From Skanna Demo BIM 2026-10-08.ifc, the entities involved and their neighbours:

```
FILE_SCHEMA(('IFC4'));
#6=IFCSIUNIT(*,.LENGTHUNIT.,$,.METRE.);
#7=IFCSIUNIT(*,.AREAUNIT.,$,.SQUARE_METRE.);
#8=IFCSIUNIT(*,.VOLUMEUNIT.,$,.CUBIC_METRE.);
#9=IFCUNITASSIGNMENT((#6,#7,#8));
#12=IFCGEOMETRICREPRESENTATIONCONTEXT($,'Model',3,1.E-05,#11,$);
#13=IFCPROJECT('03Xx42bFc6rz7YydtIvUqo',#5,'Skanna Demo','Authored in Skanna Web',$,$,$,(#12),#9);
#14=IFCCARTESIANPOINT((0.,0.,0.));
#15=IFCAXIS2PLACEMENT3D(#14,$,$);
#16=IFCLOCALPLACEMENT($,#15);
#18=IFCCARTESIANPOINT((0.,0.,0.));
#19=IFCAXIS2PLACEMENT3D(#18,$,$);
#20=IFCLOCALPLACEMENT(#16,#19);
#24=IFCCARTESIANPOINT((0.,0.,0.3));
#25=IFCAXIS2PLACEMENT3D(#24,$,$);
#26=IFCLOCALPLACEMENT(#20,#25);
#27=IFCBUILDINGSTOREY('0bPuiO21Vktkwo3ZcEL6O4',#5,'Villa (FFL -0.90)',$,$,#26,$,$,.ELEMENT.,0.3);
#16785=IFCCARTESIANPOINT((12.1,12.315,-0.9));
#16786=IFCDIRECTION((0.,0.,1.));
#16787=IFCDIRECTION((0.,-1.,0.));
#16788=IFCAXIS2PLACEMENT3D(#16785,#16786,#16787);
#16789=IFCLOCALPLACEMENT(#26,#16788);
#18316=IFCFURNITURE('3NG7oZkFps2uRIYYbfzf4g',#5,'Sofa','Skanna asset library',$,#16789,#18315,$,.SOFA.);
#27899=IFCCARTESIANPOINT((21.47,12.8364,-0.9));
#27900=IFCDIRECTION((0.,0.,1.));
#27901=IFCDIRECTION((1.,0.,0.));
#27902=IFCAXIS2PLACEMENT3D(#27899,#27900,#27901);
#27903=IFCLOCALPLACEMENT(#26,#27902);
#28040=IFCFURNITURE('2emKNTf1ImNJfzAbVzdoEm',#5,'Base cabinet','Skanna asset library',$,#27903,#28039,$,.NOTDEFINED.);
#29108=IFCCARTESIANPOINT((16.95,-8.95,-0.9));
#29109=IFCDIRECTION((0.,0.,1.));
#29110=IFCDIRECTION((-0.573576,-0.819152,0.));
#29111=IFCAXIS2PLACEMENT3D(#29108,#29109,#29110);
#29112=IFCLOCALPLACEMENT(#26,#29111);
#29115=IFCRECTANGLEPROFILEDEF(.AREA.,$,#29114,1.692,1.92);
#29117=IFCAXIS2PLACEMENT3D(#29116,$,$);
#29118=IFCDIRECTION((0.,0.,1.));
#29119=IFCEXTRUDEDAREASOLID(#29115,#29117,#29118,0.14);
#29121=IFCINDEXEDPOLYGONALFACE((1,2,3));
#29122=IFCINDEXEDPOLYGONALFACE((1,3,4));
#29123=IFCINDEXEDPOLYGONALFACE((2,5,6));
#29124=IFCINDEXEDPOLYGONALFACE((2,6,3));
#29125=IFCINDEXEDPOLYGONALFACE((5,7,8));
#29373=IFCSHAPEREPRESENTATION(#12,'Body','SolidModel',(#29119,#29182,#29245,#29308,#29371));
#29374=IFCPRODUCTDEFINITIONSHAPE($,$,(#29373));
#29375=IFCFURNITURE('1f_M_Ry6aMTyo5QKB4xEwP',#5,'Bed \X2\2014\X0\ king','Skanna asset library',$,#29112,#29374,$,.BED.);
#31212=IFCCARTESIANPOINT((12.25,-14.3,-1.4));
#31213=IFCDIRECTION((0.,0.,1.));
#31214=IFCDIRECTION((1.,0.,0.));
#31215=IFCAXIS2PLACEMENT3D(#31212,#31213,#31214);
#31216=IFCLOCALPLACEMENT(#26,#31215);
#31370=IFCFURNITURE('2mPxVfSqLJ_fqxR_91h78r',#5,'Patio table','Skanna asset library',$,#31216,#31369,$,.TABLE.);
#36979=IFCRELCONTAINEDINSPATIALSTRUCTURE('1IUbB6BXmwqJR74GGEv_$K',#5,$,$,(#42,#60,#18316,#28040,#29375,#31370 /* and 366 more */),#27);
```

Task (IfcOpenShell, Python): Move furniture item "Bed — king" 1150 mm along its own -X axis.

```python
import ifcopenshell
import ifcopenshell.api.geometry
import ifcopenshell.util.placement
import ifcopenshell.util.unit

model = ifcopenshell.open("Skanna Demo BIM 2026-10-08.ifc")
unit_scale = ifcopenshell.util.unit.calculate_unit_scale(model)

item = model.by_id(29375)
matrix = ifcopenshell.util.placement.get_local_placement(item.ObjectPlacement)
matrix[:3, 3] -= matrix[:3, 0] * 1.15 / unit_scale
ifcopenshell.api.geometry.edit_object_placement(model, product=item, matrix=matrix, is_si=False)

print(ifcopenshell.util.placement.get_local_placement(item.ObjectPlacement).round(3) + 0.0)

model.write("Skanna Demo BIM 2026-10-08_v2.ifc")
```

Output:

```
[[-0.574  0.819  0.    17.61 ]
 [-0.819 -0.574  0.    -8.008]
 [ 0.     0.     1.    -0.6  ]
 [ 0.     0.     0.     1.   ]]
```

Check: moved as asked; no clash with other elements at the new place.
